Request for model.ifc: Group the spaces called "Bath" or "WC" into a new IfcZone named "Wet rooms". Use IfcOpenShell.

First a look at what the model holds.

```python
import ifcopenshell

model = ifcopenshell.open("model.ifc")
print(model.schema)
seen = {}
for space in model.by_type("IfcSpace"):
    seen[space.LongName] = seen.get(space.LongName, 0) + 1
for name, count in sorted(seen.items(), key=str):
    print(count, "x", name)
print("zones:", [z.Name for z in model.by_type("IfcZone")][:20])
```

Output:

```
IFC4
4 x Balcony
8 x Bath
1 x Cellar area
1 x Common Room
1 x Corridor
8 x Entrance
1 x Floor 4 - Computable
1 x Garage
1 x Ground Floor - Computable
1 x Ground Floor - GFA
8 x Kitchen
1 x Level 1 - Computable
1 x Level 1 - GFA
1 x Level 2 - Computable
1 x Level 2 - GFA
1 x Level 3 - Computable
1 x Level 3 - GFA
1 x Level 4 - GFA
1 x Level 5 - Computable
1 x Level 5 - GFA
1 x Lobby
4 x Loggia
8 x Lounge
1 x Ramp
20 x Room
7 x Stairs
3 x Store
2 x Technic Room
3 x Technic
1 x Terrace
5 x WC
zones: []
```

```python
import ifcopenshell
import ifcopenshell.api.group
import ifcopenshell.api.root

model = ifcopenshell.open("model.ifc")

names = {"Bath", "WC"}
spaces = [s for s in model.by_type("IfcSpace") if s.LongName in names]

zone = ifcopenshell.api.root.create_entity(model, ifc_class="IfcZone", name="Wet rooms")
ifcopenshell.api.group.assign_group(model, products=spaces, group=zone)
print(len(spaces), "spaces in", zone.Name)

model.write("model_rev.ifc")
```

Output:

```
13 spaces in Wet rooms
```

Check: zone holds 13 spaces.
